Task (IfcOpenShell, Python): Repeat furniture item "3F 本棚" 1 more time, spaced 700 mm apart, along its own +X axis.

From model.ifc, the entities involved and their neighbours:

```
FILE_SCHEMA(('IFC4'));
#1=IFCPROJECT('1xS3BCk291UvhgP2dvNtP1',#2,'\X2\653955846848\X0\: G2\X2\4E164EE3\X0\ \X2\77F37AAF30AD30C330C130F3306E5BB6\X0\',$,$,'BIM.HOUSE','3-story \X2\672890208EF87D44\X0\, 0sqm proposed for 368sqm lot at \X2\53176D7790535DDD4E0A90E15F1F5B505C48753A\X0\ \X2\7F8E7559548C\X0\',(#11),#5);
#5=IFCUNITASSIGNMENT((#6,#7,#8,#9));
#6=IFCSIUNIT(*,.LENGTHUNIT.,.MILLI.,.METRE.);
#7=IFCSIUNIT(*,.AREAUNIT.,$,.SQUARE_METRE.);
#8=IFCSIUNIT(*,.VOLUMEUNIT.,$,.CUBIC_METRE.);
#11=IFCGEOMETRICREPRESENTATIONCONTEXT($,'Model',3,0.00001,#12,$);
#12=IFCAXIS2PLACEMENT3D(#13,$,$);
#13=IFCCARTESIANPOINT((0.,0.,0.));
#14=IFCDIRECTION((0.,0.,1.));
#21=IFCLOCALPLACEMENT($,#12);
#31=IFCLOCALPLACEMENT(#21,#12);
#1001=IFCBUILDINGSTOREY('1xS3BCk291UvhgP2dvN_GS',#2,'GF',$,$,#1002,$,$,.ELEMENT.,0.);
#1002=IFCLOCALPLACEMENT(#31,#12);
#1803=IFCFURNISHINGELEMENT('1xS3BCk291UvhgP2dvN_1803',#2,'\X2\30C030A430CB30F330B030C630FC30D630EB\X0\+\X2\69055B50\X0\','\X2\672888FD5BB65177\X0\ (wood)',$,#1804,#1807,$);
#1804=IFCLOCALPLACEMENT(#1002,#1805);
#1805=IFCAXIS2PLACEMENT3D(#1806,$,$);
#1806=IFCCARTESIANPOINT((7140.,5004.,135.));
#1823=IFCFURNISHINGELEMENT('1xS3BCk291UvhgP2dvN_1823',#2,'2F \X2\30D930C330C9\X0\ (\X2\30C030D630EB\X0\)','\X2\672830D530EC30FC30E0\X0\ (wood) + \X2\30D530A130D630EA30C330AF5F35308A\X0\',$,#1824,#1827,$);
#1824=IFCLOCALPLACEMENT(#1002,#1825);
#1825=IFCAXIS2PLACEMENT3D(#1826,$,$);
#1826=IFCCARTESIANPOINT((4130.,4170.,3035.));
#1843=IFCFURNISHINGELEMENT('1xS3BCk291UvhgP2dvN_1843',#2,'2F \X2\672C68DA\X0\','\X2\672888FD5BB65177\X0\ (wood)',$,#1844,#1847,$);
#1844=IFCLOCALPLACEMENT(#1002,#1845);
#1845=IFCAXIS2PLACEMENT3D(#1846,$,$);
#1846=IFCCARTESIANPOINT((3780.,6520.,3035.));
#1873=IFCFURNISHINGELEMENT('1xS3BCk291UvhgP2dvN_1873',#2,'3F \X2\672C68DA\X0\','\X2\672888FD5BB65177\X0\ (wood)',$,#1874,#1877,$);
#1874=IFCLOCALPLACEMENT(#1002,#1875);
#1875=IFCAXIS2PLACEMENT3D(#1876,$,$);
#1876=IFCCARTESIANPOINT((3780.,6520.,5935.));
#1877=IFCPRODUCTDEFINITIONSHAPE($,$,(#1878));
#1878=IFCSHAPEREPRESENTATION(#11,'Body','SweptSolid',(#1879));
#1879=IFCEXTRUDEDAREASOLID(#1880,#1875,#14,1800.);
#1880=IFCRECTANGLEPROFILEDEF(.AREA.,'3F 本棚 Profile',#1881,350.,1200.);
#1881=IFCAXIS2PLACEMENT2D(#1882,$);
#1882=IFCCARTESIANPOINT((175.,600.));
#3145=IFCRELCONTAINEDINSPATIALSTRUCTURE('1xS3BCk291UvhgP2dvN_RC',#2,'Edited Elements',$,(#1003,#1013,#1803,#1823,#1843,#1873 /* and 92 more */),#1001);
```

```python
import ifcopenshell
import ifcopenshell.api.geometry
import ifcopenshell.api.root
import ifcopenshell.util.element
import ifcopenshell.util.placement
import ifcopenshell.util.unit

model = ifcopenshell.open("model.ifc")
unit_scale = ifcopenshell.util.unit.calculate_unit_scale(model)


def reuse_history(source, copy):
    """copy_class also copies each property set's owner history, people and application; keep the originals."""
    for rel in copy.IsDefinedBy:
        if rel.is_a("IfcRelDefinesByProperties") and (history := rel.RelatingPropertyDefinition.OwnerHistory):
            rel.RelatingPropertyDefinition.OwnerHistory = source.OwnerHistory
            ifcopenshell.util.element.remove_deep2(model, history)


source = model.by_id(1873)
base = ifcopenshell.util.placement.get_local_placement(source.ObjectPlacement)
step = base[:3, 0] * 0.7 / unit_scale

for i in range(1, 2):
    copy = ifcopenshell.api.root.copy_class(model, product=source)
    copy.Representation = ifcopenshell.util.element.copy_deep(
        model, source.Representation, exclude=["IfcGeometricRepresentationContext", "IfcRepresentationMap"]
    )
    reuse_history(source, copy)
    matrix = base.copy()
    matrix[:3, 3] += i * step
    print("added at", matrix[:3, 3].round(3) + 0.0)
    ifcopenshell.api.geometry.edit_object_placement(model, product=copy, matrix=matrix, is_si=False)

model.write("model_updated.ifc")
```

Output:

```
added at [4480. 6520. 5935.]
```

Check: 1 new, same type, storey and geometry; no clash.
